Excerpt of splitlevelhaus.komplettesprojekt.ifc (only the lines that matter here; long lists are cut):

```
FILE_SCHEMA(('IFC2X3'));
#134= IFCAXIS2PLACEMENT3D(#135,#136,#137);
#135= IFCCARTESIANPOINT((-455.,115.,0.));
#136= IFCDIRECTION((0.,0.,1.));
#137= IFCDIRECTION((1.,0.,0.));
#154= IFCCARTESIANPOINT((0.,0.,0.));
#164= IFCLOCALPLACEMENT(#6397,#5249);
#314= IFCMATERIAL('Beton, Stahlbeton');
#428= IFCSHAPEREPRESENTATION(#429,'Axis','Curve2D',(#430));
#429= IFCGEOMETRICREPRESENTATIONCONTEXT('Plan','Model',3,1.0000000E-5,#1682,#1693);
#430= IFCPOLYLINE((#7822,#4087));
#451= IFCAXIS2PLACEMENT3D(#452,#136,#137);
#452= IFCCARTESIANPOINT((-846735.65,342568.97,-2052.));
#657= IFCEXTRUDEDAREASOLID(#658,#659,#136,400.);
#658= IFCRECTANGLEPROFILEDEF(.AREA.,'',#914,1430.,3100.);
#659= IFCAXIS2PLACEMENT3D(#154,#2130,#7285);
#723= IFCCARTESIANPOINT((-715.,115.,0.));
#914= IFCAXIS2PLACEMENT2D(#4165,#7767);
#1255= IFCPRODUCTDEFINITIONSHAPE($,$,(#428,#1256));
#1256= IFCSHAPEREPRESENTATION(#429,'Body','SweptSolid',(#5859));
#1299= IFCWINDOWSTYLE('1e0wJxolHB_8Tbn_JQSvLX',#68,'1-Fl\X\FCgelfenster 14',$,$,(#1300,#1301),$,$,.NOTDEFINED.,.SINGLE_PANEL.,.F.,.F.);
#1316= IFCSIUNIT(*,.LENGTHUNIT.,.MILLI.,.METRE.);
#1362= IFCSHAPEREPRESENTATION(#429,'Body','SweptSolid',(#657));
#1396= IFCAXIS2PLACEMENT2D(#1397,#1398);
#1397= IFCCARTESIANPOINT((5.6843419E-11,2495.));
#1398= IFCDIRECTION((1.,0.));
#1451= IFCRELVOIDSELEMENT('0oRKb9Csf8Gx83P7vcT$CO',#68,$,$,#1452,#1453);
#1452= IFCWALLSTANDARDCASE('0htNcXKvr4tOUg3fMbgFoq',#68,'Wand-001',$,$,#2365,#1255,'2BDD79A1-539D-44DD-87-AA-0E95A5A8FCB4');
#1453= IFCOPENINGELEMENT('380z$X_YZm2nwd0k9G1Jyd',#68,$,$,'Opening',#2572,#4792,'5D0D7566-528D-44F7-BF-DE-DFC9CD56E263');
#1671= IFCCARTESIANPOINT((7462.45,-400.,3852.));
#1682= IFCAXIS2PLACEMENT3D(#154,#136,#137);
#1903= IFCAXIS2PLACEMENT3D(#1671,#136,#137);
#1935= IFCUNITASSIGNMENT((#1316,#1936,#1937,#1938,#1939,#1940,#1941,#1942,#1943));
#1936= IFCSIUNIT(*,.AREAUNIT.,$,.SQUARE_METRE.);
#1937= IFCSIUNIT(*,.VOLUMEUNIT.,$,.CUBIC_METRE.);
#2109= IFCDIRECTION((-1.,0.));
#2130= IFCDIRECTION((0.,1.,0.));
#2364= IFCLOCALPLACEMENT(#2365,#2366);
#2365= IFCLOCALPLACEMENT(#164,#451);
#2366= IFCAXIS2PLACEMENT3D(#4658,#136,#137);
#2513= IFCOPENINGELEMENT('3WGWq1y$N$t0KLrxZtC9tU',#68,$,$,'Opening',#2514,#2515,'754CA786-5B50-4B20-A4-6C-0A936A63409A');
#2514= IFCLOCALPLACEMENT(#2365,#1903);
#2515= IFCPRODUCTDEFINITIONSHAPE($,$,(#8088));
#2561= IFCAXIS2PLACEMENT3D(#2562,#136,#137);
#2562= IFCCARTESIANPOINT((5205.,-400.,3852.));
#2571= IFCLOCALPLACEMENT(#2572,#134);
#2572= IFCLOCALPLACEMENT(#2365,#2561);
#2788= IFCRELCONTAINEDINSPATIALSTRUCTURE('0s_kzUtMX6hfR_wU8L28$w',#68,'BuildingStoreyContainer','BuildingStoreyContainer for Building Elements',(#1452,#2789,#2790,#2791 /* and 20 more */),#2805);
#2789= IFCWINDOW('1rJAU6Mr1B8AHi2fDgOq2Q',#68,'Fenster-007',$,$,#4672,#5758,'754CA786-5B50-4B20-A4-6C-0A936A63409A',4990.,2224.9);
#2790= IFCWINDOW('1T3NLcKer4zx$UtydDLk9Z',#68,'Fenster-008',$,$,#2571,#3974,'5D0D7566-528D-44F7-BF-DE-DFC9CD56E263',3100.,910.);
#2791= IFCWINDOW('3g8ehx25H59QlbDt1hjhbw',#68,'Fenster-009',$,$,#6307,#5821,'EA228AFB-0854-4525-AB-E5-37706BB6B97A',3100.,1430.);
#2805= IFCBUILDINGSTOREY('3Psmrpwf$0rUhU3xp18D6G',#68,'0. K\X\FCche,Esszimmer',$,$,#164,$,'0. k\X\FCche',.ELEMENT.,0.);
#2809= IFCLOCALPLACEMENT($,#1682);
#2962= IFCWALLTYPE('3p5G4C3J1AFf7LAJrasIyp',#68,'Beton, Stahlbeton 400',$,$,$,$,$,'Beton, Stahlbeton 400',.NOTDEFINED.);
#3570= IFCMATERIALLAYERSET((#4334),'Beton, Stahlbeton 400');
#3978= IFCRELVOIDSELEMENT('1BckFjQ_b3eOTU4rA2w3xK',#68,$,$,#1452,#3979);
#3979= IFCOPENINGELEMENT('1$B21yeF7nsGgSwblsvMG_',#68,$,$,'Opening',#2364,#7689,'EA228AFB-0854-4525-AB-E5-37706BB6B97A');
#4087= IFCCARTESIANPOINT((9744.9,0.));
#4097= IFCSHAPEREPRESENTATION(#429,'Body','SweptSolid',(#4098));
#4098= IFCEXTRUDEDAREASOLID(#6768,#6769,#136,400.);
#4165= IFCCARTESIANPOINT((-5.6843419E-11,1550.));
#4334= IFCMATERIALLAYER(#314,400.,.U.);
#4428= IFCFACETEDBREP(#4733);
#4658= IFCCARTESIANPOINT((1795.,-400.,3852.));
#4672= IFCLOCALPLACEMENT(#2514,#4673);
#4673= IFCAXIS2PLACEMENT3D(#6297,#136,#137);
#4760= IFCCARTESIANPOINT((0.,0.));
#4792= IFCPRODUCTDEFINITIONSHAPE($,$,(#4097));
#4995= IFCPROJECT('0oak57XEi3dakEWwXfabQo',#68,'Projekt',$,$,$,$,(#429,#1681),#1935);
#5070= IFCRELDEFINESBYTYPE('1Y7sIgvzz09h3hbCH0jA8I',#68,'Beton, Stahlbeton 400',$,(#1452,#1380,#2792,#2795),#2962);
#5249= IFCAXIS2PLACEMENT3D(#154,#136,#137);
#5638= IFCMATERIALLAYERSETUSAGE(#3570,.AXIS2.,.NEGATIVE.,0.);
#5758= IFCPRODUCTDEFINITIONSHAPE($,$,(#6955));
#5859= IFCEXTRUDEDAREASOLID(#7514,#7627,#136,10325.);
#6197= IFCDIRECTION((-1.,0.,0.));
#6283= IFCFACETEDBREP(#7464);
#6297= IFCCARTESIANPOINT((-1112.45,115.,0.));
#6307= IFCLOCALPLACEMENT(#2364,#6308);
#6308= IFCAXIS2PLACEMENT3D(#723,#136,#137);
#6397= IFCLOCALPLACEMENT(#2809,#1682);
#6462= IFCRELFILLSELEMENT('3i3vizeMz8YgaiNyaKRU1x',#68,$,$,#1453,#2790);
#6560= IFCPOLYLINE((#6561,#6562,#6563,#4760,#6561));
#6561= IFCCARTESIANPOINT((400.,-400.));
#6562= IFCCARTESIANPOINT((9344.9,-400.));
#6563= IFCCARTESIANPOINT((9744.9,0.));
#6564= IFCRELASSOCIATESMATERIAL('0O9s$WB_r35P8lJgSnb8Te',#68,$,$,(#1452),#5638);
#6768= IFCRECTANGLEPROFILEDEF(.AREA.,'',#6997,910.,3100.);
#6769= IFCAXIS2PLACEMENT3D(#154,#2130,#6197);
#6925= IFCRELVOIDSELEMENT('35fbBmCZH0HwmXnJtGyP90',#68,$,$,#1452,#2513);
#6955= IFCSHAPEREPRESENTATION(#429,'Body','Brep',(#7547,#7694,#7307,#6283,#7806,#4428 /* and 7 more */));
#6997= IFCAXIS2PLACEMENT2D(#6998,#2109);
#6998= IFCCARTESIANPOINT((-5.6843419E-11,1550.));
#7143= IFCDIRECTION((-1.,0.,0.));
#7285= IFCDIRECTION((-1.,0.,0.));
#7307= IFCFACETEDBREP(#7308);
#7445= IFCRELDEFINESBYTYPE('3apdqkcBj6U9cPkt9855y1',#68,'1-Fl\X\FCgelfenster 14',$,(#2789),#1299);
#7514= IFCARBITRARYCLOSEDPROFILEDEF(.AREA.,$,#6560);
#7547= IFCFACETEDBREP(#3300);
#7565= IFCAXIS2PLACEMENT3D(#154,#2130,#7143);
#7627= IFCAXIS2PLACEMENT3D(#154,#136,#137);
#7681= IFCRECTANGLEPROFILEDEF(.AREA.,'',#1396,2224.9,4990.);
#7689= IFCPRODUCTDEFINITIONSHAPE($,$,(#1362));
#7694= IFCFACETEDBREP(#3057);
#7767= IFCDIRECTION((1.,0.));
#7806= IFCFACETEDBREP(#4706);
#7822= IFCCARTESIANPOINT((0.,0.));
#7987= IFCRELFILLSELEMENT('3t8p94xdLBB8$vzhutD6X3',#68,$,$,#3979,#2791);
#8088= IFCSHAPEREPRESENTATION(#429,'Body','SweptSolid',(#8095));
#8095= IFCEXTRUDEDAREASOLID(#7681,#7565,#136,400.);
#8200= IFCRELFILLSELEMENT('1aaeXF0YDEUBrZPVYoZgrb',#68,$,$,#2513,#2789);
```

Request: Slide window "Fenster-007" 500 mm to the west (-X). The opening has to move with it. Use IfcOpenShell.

```python
import ifcopenshell
import ifcopenshell.api.geometry
import ifcopenshell.util.placement
import ifcopenshell.util.unit

model = ifcopenshell.open("splitlevelhaus.komplettesprojekt.ifc")
unit_scale = ifcopenshell.util.unit.calculate_unit_scale(model)

window = model.by_id(2789)
opening = window.FillsVoids[0].RelatingOpeningElement
wall = opening.VoidsElements[0].RelatingBuildingElement

wall_matrix = ifcopenshell.util.placement.get_local_placement(wall.ObjectPlacement)
shift = wall_matrix[:3, 0] * -0.5 / unit_scale
before = ifcopenshell.util.placement.get_local_placement(window.ObjectPlacement)[:3, 3].copy()

# The window is placed relative to its opening, so it follows when the opening moves.
matrix = ifcopenshell.util.placement.get_local_placement(opening.ObjectPlacement)
matrix[:3, 3] += shift
ifcopenshell.api.geometry.edit_object_placement(
    model, product=opening, matrix=matrix, is_si=False, should_transform_children=True
)

after = ifcopenshell.util.placement.get_local_placement(window.ObjectPlacement)[:3, 3]
print("window moved by", (after - before).round(3) + 0.0)

model.write("splitlevelhaus.komplettesprojekt_v2.ifc")
```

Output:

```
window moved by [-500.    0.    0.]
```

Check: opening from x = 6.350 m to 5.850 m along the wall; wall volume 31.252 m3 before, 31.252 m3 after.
